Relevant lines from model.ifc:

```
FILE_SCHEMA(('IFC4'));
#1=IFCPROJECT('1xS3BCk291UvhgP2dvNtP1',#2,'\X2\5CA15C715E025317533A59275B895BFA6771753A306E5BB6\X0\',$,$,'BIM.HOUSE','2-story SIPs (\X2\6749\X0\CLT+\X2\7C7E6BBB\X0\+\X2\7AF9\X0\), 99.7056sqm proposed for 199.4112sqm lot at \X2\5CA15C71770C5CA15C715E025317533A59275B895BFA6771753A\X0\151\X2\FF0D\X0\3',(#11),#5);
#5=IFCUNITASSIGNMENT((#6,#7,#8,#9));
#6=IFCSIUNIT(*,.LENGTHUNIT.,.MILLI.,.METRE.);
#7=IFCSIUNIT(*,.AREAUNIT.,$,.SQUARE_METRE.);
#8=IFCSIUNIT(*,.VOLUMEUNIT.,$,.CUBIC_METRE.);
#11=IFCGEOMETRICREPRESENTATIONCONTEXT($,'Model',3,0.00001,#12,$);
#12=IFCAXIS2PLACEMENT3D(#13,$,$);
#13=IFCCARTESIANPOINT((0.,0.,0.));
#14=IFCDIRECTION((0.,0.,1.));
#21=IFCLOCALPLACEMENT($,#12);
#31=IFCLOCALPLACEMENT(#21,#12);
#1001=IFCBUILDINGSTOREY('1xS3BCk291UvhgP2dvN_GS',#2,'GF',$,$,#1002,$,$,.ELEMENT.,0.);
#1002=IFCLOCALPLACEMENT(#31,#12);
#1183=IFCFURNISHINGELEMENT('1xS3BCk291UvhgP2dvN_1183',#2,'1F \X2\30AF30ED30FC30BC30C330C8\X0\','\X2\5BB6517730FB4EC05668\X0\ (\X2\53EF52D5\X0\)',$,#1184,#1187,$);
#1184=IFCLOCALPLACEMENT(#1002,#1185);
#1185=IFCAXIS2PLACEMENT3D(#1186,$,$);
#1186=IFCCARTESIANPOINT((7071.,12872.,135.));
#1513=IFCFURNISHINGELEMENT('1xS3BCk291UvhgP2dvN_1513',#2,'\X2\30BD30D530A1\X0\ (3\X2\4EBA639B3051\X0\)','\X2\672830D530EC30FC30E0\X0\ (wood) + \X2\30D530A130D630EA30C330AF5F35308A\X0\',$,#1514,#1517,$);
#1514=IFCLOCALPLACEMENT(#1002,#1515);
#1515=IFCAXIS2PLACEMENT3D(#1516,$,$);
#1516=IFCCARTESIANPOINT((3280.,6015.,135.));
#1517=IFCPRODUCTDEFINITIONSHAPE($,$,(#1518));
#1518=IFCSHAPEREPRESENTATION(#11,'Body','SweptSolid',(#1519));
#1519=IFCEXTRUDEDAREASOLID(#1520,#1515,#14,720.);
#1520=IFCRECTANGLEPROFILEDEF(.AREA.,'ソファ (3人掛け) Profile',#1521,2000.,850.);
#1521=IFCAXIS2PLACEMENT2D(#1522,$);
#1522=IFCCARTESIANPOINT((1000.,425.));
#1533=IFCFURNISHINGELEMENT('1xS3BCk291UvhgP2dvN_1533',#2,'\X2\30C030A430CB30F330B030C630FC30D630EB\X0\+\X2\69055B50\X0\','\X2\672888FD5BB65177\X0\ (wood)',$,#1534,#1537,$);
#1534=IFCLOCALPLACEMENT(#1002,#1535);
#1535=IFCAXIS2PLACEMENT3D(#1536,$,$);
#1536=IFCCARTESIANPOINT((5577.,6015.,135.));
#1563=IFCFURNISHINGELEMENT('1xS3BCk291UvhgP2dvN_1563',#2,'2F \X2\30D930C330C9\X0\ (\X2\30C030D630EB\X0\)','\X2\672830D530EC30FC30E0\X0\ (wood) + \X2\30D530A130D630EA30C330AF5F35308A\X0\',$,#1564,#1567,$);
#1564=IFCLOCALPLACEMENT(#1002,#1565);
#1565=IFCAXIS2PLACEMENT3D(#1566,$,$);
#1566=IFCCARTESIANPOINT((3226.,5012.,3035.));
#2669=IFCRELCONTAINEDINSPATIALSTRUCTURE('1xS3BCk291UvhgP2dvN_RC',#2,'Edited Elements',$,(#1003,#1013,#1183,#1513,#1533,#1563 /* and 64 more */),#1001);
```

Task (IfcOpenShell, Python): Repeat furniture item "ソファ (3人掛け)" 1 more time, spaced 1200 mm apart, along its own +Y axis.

```python
import ifcopenshell
import ifcopenshell.api.geometry
import ifcopenshell.api.root
import ifcopenshell.util.element
import ifcopenshell.util.placement

model = ifcopenshell.open("model.ifc")


def reuse_history(source, copy):
    """copy_class also copies each property set's owner history, people and application; keep the originals."""
    for rel in copy.IsDefinedBy:
        if rel.is_a("IfcRelDefinesByProperties") and (history := rel.RelatingPropertyDefinition.OwnerHistory):
            rel.RelatingPropertyDefinition.OwnerHistory = source.OwnerHistory
            ifcopenshell.util.element.remove_deep2(model, history)


source = model.by_guid("1xS3BCk291UvhgP2dvN_1513")
base = ifcopenshell.util.placement.get_local_placement(source.ObjectPlacement)
step = base[:3, 1] * 1200.0

for i in range(1, 2):
    copy = ifcopenshell.api.root.copy_class(model, product=source)
    copy.Representation = ifcopenshell.util.element.copy_deep(
        model, source.Representation, exclude=["IfcGeometricRepresentationContext", "IfcRepresentationMap"]
    )
    reuse_history(source, copy)
    matrix = base.copy()
    matrix[:3, 3] += i * step
    print("added at", matrix[:3, 3].round(3) + 0.0)
    ifcopenshell.api.geometry.edit_object_placement(model, product=copy, matrix=matrix, is_si=False)

model.write("model_edited.ifc")
```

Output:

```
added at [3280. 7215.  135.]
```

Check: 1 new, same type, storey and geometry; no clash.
